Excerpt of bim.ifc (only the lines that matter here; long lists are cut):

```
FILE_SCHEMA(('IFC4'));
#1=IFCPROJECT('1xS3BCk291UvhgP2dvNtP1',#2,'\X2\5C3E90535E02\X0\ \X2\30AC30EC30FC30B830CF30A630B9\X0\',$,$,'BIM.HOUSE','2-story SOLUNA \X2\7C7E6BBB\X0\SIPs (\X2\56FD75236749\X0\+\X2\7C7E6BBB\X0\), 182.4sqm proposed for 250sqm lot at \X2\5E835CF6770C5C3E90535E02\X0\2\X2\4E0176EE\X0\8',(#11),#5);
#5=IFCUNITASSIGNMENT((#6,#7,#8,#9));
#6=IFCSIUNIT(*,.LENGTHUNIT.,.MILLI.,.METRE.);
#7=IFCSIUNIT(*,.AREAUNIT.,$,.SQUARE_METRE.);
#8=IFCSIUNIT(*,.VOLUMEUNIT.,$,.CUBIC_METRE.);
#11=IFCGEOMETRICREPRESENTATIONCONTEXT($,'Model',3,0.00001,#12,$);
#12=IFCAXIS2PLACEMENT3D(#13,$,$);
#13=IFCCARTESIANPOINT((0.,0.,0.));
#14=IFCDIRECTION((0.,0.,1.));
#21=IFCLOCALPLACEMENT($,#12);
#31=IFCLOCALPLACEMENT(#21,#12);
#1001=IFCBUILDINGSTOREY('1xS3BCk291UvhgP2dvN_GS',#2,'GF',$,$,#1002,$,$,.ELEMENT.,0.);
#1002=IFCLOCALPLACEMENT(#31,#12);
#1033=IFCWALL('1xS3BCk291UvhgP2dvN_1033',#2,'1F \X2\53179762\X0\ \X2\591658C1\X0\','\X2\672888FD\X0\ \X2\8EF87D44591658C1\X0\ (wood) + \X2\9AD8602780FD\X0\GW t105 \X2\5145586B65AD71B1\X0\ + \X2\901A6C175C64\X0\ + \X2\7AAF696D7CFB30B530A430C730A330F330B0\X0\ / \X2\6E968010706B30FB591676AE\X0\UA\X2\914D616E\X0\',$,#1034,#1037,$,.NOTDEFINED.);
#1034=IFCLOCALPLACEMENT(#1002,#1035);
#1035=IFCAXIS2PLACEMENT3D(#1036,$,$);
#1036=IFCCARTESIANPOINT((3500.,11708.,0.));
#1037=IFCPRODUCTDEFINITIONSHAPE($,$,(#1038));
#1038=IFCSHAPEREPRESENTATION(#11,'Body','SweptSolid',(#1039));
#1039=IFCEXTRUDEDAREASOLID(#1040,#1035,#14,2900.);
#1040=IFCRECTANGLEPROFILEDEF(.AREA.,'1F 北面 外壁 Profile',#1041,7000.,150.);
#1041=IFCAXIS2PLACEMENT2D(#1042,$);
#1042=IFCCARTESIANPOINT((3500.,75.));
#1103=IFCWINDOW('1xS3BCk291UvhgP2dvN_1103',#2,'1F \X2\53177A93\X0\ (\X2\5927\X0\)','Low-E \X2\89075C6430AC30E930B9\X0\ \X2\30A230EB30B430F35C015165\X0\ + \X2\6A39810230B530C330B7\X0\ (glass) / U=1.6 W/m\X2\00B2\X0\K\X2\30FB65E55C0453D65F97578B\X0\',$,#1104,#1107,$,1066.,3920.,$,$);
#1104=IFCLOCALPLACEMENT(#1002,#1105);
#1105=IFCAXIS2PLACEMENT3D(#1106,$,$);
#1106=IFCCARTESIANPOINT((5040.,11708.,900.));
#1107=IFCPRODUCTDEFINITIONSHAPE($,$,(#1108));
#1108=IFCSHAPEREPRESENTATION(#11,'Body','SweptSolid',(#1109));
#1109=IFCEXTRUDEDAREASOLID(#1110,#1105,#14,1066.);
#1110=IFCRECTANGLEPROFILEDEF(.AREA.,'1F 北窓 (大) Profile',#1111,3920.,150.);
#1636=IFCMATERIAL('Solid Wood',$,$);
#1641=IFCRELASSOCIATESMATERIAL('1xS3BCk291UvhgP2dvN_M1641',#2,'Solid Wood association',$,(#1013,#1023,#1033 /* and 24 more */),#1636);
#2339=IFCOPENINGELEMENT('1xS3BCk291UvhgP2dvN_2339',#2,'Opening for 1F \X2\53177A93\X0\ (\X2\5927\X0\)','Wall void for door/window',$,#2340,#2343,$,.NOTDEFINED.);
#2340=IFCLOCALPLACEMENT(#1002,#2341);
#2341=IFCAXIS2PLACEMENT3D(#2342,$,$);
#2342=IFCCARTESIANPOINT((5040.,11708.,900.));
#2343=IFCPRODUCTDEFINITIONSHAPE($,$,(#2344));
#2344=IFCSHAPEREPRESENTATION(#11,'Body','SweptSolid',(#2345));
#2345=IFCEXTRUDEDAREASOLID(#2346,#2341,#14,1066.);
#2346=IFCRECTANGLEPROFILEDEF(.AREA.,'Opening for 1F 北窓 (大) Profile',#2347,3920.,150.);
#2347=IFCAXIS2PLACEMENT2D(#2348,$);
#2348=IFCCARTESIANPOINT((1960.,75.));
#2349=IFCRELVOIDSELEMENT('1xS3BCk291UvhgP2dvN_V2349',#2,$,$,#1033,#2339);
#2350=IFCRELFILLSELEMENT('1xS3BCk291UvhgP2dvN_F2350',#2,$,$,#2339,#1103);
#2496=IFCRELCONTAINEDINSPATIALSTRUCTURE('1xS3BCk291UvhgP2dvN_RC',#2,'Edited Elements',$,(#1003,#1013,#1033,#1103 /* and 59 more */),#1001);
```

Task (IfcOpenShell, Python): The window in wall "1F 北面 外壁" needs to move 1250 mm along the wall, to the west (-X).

```python
import ifcopenshell
import ifcopenshell.api.geometry
import ifcopenshell.util.placement
import ifcopenshell.util.unit

model = ifcopenshell.open("bim.ifc")
unit_scale = ifcopenshell.util.unit.calculate_unit_scale(model)

window = model.by_id(1103)
opening = window.FillsVoids[0].RelatingOpeningElement
wall = opening.VoidsElements[0].RelatingBuildingElement

wall_matrix = ifcopenshell.util.placement.get_local_placement(wall.ObjectPlacement)
shift = wall_matrix[:3, 0] * -1.25 / unit_scale
before = ifcopenshell.util.placement.get_local_placement(window.ObjectPlacement)[:3, 3].copy()

# The window is not placed relative to its opening, so move both.
for product in (opening, window):
    matrix = ifcopenshell.util.placement.get_local_placement(product.ObjectPlacement)
    matrix[:3, 3] += shift
    ifcopenshell.api.geometry.edit_object_placement(model, product=product, matrix=matrix, is_si=False)

after = ifcopenshell.util.placement.get_local_placement(window.ObjectPlacement)[:3, 3]
print("window moved by", (after - before).round(3) + 0.0)

model.write("bim_edited.ifc")
```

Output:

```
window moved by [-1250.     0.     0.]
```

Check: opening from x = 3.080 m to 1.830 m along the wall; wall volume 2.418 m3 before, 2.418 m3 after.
